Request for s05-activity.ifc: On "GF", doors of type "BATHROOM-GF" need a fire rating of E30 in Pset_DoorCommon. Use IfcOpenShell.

First a look at what the model holds.

```python
import ifcopenshell
import ifcopenshell.util.element

model = ifcopenshell.open("s05-activity.ifc")
print(model.schema)
storey = next(s for s in model.by_type("IfcBuildingStorey") if s.Name == "GF")
doors = [e for e in ifcopenshell.util.element.get_decomposition(storey) if e.is_a("IfcDoor")]
seen = {}
for e in doors:
    element_type = ifcopenshell.util.element.get_type(e)
    key = (element_type.Name if element_type != e and element_type else None, ifcopenshell.util.element.get_pset(e, "Pset_DoorCommon", "FireRating"))
    seen[key] = seen.get(key, 0) + 1
for (name, value), count in sorted(seen.items(), key=str):
    print(count, "x", name, "|", value)
```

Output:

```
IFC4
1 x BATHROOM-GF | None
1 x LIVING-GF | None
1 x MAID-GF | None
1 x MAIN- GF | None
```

```python
import ifcopenshell
import ifcopenshell.api.pset
import ifcopenshell.util.element

model = ifcopenshell.open("s05-activity.ifc")

storey = next(s for s in model.by_type("IfcBuildingStorey") if s.Name == "GF")
doors = [e for e in ifcopenshell.util.element.get_decomposition(storey) if e.is_a("IfcDoor")]

count = 0
for e in doors:
    element_type = ifcopenshell.util.element.get_type(e)
    if element_type in (None, e) or element_type.Name != "BATHROOM-GF":
        continue
    # add_pset returns the element's existing set when there is one.
    pset = ifcopenshell.api.pset.add_pset(model, product=e, name="Pset_DoorCommon")
    ifcopenshell.api.pset.edit_pset(model, pset=pset, properties={"FireRating": "E30"})
    count += 1

print(count, "doors updated")

model.write("s05-activity-out.ifc")
```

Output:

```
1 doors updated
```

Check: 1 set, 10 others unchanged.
